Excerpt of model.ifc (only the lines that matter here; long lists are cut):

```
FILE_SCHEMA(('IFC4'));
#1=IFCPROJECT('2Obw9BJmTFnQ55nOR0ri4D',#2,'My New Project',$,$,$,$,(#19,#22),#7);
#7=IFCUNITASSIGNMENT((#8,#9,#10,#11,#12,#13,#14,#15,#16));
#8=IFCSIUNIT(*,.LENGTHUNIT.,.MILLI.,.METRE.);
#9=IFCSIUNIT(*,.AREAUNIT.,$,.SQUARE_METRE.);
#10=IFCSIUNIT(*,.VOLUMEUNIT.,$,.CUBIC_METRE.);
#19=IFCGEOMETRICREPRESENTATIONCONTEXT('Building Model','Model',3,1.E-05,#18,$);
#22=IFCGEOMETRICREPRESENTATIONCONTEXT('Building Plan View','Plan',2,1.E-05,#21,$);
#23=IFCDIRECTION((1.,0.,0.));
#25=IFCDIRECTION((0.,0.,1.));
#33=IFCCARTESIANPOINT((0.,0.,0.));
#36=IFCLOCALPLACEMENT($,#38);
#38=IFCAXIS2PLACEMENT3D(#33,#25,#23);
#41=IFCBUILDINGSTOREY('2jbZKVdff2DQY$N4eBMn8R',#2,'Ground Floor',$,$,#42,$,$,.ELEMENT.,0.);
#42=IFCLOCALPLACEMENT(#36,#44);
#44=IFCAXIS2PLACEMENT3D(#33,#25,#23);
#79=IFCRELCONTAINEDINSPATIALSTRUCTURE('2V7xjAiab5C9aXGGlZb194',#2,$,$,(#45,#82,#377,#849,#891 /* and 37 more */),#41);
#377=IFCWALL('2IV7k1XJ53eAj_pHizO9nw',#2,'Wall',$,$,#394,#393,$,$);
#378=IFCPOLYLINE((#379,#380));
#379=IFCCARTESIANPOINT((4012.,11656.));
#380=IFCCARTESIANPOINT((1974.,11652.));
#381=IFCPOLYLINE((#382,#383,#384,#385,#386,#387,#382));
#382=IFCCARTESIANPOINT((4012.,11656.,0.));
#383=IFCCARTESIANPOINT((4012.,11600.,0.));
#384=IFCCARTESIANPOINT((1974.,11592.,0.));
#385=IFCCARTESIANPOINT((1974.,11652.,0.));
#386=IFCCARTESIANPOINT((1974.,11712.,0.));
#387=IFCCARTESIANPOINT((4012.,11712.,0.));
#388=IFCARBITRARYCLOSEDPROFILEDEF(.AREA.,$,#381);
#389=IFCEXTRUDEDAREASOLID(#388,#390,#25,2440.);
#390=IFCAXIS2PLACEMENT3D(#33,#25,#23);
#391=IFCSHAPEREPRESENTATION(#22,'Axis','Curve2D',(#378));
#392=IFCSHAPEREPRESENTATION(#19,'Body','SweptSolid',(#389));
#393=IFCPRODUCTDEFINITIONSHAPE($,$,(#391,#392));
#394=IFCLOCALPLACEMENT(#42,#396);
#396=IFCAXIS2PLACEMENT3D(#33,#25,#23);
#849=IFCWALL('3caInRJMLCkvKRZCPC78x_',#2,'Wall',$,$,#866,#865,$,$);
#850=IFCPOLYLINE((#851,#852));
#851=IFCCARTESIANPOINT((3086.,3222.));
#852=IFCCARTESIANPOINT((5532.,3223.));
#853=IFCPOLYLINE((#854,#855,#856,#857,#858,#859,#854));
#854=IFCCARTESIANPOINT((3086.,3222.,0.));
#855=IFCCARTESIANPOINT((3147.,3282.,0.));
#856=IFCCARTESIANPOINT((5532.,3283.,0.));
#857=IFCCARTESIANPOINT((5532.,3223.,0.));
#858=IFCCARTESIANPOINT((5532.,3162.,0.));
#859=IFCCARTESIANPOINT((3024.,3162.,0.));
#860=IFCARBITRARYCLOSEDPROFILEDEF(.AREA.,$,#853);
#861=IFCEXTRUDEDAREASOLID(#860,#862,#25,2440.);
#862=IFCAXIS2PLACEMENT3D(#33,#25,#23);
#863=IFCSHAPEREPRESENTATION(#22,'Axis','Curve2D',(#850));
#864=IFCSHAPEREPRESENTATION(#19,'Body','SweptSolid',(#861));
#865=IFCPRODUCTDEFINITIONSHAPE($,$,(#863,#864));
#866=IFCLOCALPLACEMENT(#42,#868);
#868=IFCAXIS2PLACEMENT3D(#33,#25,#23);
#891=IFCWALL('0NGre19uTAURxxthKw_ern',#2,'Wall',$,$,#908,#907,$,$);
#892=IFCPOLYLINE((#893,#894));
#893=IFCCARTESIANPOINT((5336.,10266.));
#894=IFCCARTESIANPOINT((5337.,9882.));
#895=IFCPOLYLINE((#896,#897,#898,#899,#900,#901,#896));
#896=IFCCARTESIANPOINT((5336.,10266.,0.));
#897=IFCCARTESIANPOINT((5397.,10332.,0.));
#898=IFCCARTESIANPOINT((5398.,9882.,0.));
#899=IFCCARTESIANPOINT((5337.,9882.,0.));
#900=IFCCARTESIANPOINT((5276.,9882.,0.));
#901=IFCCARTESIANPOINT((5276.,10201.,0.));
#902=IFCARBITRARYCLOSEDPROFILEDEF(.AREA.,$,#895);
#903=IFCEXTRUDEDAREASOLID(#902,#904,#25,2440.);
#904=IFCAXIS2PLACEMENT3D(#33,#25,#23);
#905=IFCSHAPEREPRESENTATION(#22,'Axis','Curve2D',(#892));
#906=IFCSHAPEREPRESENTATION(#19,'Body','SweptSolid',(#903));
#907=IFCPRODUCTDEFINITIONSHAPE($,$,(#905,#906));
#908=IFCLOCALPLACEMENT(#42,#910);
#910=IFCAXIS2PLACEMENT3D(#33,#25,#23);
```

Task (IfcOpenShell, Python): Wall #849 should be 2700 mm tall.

```python
import ifcopenshell
import ifcopenshell.geom
import ifcopenshell.util.shape

model = ifcopenshell.open("model.ifc")
settings = ifcopenshell.geom.settings()


def volume(element):
    """Net volume in cubic metres, openings subtracted."""
    shape = ifcopenshell.geom.create_shape(settings, element)
    return ifcopenshell.util.shape.get_volume(shape.geometry)


wall = model.by_guid("3caInRJMLCkvKRZCPC78x_")
before = volume(wall)

body = next(r for r in wall.Representation.Representations if r.RepresentationIdentifier == "Body")
solid = body.Items[0]
old_height = solid.Depth
solid.Depth = 2700.0
after = volume(wall)

print(f"height {old_height:g} -> {solid.Depth:g}, volume {before:.3f} -> {after:.3f} m3")

model.write("model-out.ifc")
```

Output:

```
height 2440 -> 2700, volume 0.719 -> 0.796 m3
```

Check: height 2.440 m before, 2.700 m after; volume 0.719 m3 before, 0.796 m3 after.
